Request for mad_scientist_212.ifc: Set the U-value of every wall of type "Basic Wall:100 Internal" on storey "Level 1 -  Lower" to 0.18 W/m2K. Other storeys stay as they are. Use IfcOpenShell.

First a look at what the model holds.

```python
import ifcopenshell
import ifcopenshell.util.element

model = ifcopenshell.open("mad_scientist_212.ifc")
print(model.schema)
storey = next(s for s in model.by_type("IfcBuildingStorey") if s.Name == "Level 1 -  Lower")
walls = [e for e in ifcopenshell.util.element.get_decomposition(storey) if e.is_a("IfcWall")]
seen = {}
for e in walls:
    element_type = ifcopenshell.util.element.get_type(e)
    key = (element_type.Name if element_type != e and element_type else None, ifcopenshell.util.element.get_pset(e, "Pset_WallCommon", "ThermalTransmittance"))
    seen[key] = seen.get(key, 0) + 1
for (name, value), count in sorted(seen.items(), key=str):
    print(count, "x", name, "|", value)
```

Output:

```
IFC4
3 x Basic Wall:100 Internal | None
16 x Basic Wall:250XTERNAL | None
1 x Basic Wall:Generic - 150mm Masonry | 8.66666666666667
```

```python
import ifcopenshell
import ifcopenshell.api.pset
import ifcopenshell.util.element

model = ifcopenshell.open("mad_scientist_212.ifc")

storey = next(s for s in model.by_type("IfcBuildingStorey") if s.Name == "Level 1 -  Lower")
walls = [e for e in ifcopenshell.util.element.get_decomposition(storey) if e.is_a("IfcWall")]

count = 0
for e in walls:
    element_type = ifcopenshell.util.element.get_type(e)
    if element_type in (None, e) or element_type.Name != "Basic Wall:100 Internal":
        continue
    # add_pset returns the element's existing set when there is one.
    pset = ifcopenshell.api.pset.add_pset(model, product=e, name="Pset_WallCommon")
    ifcopenshell.api.pset.edit_pset(model, pset=pset, properties={"ThermalTransmittance": 0.18})
    count += 1

print(count, "walls updated")

model.write("mad_scientist_212_edited.ifc")
```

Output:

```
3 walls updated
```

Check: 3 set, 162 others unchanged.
